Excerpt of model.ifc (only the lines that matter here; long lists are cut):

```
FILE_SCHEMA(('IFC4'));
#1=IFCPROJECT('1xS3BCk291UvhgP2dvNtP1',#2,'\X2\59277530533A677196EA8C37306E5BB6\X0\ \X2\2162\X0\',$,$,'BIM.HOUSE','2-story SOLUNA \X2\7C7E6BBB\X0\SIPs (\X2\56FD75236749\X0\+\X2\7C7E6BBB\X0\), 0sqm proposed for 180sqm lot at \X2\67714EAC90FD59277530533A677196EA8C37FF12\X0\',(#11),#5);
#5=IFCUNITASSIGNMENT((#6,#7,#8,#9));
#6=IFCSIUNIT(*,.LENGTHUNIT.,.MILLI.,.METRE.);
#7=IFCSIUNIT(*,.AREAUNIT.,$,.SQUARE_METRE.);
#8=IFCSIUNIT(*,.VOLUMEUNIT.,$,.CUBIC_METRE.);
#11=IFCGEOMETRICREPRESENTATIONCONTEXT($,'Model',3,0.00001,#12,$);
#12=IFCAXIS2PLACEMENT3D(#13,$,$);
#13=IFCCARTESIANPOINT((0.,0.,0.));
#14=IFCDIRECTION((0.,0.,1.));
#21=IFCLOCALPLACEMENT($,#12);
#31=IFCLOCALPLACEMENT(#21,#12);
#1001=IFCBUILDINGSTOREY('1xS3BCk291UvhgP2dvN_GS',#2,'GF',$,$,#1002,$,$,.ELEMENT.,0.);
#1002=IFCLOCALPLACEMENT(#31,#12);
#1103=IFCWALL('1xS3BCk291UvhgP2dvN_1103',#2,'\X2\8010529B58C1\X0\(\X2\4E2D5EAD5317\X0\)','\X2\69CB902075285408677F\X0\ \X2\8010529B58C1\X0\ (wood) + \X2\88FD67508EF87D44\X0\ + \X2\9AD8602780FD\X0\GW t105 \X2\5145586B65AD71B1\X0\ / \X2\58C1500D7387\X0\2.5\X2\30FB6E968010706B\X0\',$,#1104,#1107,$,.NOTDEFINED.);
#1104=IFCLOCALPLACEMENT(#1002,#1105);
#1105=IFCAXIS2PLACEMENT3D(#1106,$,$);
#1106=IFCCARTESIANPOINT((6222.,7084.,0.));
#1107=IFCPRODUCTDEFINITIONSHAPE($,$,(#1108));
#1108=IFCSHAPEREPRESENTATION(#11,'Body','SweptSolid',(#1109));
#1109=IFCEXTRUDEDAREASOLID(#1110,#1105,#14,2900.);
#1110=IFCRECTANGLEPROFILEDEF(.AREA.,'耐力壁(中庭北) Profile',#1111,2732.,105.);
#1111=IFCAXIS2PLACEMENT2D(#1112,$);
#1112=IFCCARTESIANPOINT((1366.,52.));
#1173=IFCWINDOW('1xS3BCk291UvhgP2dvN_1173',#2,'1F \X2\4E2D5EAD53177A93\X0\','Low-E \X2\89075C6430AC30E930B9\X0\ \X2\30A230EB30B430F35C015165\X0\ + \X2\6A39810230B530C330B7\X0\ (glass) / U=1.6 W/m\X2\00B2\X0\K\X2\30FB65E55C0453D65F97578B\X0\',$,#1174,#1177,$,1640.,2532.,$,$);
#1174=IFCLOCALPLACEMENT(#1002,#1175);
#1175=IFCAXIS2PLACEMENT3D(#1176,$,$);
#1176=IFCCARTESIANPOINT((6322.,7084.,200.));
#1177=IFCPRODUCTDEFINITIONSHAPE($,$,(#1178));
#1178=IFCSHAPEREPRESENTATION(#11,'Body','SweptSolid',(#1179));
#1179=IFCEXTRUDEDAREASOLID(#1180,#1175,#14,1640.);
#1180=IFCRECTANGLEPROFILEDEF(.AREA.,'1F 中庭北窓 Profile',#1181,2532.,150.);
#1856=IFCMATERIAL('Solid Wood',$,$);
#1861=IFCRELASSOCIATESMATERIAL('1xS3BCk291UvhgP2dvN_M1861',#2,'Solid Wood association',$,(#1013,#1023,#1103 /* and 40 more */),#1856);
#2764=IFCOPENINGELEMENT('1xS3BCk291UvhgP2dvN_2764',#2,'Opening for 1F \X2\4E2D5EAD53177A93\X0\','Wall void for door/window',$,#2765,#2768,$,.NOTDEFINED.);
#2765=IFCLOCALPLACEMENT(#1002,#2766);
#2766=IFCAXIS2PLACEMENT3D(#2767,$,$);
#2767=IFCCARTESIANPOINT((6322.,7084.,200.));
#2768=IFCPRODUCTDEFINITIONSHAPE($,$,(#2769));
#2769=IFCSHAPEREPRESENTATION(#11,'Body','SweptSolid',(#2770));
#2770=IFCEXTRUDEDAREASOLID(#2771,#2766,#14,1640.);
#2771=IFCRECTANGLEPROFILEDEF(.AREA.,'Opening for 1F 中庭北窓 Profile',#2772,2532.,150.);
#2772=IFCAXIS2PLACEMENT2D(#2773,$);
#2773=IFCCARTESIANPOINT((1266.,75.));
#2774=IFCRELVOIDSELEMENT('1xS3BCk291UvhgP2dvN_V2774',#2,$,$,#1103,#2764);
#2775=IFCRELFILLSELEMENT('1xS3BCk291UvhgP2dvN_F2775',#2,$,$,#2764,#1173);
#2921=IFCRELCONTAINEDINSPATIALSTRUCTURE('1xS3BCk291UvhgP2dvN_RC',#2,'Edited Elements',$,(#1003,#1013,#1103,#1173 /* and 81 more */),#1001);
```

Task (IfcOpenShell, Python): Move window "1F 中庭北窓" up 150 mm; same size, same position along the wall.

```python
import numpy as np
import ifcopenshell
import ifcopenshell.api.geometry
import ifcopenshell.util.placement
import ifcopenshell.util.unit

model = ifcopenshell.open("model.ifc")
unit_scale = ifcopenshell.util.unit.calculate_unit_scale(model)

window = model.by_guid("1xS3BCk291UvhgP2dvN_1173")
opening = window.FillsVoids[0].RelatingOpeningElement
dz = 150.0

shift = np.array([0.0, 0.0, dz])
# The window is not placed relative to its opening, so move both.
for product in (opening, window):
    matrix = ifcopenshell.util.placement.get_local_placement(product.ObjectPlacement)
    matrix[:3, 3] += shift
    ifcopenshell.api.geometry.edit_object_placement(model, product=product, matrix=matrix, is_si=False)

print(f"moved by {dz * unit_scale:+.3f} m")

model.write("model_edited.ifc")
```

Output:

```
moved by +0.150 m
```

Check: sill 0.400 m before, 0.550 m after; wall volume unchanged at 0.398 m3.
